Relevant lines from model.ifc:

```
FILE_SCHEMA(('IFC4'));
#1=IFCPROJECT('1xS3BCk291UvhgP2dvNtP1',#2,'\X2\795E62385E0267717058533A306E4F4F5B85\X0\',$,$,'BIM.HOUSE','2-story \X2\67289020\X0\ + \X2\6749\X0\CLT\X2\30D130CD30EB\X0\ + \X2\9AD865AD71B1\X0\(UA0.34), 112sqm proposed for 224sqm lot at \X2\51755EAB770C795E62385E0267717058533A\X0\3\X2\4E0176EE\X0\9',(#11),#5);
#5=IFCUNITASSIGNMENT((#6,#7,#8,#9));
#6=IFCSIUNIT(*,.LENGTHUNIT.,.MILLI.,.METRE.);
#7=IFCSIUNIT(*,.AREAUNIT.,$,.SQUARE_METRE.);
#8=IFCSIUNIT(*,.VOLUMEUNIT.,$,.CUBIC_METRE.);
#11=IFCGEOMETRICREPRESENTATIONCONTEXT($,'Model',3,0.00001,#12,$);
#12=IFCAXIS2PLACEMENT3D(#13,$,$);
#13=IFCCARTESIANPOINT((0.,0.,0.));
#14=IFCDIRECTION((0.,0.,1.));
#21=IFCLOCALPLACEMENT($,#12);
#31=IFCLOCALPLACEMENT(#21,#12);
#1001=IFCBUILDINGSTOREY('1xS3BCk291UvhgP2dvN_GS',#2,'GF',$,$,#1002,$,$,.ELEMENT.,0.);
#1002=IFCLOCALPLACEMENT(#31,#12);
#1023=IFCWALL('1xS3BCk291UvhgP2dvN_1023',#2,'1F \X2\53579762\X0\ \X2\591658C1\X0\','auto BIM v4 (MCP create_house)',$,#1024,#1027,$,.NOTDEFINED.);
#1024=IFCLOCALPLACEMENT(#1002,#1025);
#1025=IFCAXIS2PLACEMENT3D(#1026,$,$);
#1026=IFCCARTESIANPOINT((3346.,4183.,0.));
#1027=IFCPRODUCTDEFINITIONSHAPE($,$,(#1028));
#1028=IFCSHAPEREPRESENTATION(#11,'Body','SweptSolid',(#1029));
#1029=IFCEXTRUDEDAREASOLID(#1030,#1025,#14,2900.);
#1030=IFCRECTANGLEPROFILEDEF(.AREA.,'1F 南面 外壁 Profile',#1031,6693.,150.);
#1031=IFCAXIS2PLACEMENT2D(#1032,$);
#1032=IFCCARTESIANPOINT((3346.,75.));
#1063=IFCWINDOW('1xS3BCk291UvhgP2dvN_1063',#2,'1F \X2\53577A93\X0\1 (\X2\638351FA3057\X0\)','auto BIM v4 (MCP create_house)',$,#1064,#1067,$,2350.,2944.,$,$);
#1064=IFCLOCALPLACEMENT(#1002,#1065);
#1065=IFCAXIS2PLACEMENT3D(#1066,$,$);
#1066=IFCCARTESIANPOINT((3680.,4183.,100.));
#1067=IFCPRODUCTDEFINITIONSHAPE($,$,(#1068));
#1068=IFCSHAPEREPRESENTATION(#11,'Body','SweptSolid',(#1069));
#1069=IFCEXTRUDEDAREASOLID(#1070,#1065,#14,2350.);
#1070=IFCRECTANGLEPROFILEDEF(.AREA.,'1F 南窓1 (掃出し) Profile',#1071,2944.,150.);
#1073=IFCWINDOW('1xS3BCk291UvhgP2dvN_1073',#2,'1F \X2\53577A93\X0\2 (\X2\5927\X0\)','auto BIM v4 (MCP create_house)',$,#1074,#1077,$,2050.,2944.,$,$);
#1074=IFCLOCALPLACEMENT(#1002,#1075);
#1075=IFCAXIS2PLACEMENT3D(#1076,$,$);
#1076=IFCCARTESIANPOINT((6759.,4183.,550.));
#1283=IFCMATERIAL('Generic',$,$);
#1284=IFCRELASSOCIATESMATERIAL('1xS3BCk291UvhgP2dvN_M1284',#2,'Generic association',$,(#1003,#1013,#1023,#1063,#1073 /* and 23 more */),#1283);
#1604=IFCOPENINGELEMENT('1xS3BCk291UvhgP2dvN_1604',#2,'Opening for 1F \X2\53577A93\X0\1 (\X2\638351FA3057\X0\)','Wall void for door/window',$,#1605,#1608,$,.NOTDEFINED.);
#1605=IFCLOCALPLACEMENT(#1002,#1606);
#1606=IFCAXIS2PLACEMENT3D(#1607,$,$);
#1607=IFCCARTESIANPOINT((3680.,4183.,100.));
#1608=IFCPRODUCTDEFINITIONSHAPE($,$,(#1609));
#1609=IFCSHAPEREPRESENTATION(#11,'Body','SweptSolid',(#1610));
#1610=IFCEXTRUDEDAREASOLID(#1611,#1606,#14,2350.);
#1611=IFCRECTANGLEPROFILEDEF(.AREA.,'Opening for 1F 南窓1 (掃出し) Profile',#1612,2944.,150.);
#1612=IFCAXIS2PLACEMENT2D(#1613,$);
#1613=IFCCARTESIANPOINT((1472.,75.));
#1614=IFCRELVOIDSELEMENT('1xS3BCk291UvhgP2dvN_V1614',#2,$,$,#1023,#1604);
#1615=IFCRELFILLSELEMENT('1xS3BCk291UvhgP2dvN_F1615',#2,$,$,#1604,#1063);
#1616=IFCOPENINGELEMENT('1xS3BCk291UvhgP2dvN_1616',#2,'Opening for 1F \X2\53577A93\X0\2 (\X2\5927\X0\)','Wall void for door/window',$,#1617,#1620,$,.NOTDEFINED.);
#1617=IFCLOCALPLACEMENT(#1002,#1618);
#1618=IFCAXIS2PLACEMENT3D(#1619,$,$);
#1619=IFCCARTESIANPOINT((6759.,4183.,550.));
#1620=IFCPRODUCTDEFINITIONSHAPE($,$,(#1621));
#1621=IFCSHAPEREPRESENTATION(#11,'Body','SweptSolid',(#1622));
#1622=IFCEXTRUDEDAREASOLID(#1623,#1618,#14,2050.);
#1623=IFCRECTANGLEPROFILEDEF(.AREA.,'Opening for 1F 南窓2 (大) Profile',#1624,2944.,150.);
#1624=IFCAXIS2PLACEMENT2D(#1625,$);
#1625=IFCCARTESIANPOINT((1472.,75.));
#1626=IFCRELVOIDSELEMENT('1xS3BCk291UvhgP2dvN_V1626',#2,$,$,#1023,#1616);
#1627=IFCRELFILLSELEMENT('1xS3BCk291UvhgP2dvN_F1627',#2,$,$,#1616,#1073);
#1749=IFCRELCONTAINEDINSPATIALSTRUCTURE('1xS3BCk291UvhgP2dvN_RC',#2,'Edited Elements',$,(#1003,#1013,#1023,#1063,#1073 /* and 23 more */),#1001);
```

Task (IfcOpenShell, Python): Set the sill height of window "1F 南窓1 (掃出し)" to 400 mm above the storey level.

```python
import numpy as np
import ifcopenshell
import ifcopenshell.api.geometry
import ifcopenshell.geom
import ifcopenshell.util.element
import ifcopenshell.util.placement
import ifcopenshell.util.shape
import ifcopenshell.util.unit

model = ifcopenshell.open("model.ifc")
unit_scale = ifcopenshell.util.unit.calculate_unit_scale(model)

window = model.by_guid("1xS3BCk291UvhgP2dvN_1063")
opening = window.FillsVoids[0].RelatingOpeningElement
storey = ifcopenshell.util.element.get_container(window, ifc_class="IfcBuildingStorey")
level = ifcopenshell.util.placement.get_local_placement(storey.ObjectPlacement)[2, 3]

# The opening's origin need not be at the sill, so measure its lowest point.
shape = ifcopenshell.geom.create_shape(ifcopenshell.geom.settings(), opening)
bottom = ifcopenshell.util.shape.get_shape_bottom_elevation(shape, shape.geometry) / unit_scale
dz = level + 0.4 / unit_scale - bottom

shift = np.array([0.0, 0.0, dz])
# The window is not placed relative to its opening, so move both.
for product in (opening, window):
    matrix = ifcopenshell.util.placement.get_local_placement(product.ObjectPlacement)
    matrix[:3, 3] += shift
    ifcopenshell.api.geometry.edit_object_placement(model, product=product, matrix=matrix, is_si=False)

print(f"moved by {dz * unit_scale:+.3f} m")

model.write("model_rev.ifc")
```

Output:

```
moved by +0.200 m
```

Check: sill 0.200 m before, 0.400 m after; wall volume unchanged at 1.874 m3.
